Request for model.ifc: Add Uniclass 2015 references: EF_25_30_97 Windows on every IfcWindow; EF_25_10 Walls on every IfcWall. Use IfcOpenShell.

First a look at what the model holds.

```python
import ifcopenshell

model = ifcopenshell.open("model.ifc")
print(model.schema)
print("classifications:", [c.Name for c in model.by_type("IfcClassification")])
for ifc_class in ("IfcDoor", "IfcRoof", "IfcStair", "IfcWall", "IfcWindow"):
    print(ifc_class, len(model.by_type(ifc_class)))
```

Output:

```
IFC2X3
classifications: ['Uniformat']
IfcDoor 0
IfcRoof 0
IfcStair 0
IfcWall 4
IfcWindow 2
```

```python
import ifcopenshell
import ifcopenshell.api.classification

model = ifcopenshell.open("model.ifc")

# IFC2X3 requires Source and Edition and has no link from the project to the system.
system = model.create_entity("IfcClassification", Source="NBS", Edition="2015", Name="Uniclass 2015")

codes = {
    "IfcWindow": ("EF_25_30_97", "Windows"),
    "IfcWall": ("EF_25_10", "Walls"),
}
for ifc_class, (code, name) in codes.items():
    products = model.by_type(ifc_class)
    ifcopenshell.api.classification.add_reference(
        model, products=products, classification=system, identification=code, name=name
    )
    print(code, len(products))

model.write("model_v2.ifc")
```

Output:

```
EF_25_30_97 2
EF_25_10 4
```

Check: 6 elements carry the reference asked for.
